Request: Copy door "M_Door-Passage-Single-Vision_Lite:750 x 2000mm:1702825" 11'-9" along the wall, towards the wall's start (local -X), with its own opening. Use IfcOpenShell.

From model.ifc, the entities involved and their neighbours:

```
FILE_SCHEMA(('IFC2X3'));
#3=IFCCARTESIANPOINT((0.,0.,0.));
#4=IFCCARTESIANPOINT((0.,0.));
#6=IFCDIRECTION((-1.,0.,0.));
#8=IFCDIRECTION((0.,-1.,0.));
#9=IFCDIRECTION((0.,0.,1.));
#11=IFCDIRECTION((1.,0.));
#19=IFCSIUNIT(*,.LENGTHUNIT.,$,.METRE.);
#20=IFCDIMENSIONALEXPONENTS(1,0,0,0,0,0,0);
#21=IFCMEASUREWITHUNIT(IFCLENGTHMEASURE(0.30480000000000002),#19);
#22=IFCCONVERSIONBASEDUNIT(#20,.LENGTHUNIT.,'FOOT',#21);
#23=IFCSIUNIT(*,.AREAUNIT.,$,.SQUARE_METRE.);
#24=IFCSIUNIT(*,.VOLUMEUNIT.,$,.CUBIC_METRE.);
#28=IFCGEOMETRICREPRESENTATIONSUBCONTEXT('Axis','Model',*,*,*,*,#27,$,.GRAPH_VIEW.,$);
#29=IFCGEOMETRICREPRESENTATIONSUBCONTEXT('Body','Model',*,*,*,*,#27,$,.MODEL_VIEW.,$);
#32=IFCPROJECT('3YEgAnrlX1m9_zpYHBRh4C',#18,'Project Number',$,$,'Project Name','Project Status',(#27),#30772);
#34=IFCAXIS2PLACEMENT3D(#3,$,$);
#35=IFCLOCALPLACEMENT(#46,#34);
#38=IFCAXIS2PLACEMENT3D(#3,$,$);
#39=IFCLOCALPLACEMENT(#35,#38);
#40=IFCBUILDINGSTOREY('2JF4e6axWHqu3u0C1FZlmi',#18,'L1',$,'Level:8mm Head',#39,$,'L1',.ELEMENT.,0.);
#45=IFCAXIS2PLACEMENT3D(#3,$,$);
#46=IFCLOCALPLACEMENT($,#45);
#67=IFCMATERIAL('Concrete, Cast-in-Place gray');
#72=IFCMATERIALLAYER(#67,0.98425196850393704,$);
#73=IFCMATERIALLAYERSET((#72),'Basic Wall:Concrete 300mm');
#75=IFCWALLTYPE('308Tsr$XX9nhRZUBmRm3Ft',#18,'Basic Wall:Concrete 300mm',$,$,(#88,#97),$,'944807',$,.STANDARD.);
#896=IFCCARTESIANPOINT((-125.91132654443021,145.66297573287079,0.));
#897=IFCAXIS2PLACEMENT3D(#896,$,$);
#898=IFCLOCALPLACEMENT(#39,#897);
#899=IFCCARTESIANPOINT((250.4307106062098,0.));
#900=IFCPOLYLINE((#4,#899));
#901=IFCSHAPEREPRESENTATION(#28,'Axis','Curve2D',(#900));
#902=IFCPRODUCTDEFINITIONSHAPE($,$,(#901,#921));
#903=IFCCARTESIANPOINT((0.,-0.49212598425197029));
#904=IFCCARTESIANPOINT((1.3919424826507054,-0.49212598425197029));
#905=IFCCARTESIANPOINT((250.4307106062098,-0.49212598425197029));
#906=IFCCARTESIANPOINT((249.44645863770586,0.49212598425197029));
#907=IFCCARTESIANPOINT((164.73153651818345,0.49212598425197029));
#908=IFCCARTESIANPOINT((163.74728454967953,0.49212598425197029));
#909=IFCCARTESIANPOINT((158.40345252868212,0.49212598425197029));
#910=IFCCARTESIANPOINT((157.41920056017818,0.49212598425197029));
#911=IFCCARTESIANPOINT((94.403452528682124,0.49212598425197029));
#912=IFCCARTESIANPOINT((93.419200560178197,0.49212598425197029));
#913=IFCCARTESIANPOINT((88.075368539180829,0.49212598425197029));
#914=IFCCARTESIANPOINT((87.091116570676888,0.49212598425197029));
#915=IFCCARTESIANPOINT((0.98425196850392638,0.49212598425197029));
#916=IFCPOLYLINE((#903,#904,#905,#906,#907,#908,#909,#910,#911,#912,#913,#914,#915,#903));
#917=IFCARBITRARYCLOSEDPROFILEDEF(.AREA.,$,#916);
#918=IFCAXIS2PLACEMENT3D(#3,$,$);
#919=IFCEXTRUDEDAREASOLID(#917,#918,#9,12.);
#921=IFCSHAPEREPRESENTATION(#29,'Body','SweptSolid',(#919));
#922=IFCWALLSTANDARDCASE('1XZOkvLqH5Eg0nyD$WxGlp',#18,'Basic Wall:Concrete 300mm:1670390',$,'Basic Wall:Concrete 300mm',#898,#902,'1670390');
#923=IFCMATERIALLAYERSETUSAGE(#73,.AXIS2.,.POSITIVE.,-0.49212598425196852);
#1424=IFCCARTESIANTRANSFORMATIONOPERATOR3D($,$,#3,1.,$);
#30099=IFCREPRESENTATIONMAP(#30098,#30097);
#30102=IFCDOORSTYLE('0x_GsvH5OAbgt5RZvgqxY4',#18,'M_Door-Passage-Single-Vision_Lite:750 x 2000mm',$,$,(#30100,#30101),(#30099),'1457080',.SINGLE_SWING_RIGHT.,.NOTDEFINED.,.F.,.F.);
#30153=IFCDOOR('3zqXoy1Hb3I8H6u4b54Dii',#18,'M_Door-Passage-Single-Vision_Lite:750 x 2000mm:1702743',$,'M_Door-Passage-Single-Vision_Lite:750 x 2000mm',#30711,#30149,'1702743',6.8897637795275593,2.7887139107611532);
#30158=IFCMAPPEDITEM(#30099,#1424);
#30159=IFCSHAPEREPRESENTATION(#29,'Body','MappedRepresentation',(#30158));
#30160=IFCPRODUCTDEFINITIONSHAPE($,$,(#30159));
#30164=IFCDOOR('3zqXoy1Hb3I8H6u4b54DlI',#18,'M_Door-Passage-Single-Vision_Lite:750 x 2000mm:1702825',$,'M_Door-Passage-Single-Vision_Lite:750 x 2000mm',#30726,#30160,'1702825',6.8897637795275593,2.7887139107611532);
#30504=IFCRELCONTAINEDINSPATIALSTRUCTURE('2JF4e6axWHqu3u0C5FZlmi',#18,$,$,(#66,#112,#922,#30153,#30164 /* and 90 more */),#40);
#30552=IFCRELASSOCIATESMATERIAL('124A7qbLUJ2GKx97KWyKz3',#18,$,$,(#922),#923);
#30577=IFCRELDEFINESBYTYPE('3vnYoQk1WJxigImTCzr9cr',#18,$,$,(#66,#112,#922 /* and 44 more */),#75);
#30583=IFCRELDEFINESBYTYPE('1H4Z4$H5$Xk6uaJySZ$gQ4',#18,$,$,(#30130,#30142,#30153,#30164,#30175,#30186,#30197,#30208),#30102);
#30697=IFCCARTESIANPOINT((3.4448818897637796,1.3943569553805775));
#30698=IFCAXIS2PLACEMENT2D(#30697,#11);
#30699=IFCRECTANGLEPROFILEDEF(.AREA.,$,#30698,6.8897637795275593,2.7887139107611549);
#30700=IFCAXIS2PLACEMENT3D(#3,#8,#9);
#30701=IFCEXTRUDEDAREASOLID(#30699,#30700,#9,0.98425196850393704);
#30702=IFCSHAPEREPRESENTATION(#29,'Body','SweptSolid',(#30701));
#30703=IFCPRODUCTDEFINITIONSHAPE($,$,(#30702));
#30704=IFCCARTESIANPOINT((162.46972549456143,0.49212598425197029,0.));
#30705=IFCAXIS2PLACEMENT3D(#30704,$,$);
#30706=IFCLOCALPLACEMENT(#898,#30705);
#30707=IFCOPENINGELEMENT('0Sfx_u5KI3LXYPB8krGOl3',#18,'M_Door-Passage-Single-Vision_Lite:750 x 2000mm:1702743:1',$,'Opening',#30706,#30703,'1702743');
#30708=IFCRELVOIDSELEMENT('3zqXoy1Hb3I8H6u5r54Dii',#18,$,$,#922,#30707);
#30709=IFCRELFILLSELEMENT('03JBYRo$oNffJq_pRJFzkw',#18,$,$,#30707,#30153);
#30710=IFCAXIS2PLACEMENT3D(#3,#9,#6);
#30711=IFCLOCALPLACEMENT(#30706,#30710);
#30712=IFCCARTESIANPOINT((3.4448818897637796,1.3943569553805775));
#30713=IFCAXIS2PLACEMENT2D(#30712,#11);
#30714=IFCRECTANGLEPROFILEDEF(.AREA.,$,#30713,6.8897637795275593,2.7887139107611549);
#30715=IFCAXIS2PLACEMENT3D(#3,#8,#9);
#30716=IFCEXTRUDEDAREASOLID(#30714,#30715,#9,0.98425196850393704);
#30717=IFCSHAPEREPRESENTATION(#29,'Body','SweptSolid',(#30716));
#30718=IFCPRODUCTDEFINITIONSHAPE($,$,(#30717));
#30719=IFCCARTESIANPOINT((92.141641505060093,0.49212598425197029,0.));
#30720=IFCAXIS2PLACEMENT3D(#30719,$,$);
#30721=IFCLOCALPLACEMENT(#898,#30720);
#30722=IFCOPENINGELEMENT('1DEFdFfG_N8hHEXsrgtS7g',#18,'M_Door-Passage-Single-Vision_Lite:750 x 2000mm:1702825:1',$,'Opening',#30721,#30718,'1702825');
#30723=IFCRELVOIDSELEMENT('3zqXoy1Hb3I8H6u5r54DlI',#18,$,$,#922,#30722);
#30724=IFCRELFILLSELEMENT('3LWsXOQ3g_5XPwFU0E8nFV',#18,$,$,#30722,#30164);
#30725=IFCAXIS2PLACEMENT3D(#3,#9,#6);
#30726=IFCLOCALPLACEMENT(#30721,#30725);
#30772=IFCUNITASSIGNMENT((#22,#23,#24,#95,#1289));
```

```python
import ifcopenshell
import ifcopenshell.api.feature
import ifcopenshell.api.geometry
import ifcopenshell.api.root
import ifcopenshell.geom
import ifcopenshell.util.element
import ifcopenshell.util.placement
import ifcopenshell.util.shape
import ifcopenshell.util.unit

model = ifcopenshell.open("model.ifc")
unit_scale = ifcopenshell.util.unit.calculate_unit_scale(model)
settings = ifcopenshell.geom.settings()


def volume(element):
    """Net volume in cubic metres, openings subtracted."""
    shape = ifcopenshell.geom.create_shape(settings, element)
    return ifcopenshell.util.shape.get_volume(shape.geometry)


def reuse_history(source, copy):
    """copy_class also copies each property set's owner history, people and application; keep the originals."""
    for rel in copy.IsDefinedBy:
        if rel.is_a("IfcRelDefinesByProperties") and (history := rel.RelatingPropertyDefinition.OwnerHistory):
            rel.RelatingPropertyDefinition.OwnerHistory = source.OwnerHistory
            ifcopenshell.util.element.remove_deep2(model, history)


door = model.by_id(30164)
opening = door.FillsVoids[0].RelatingOpeningElement
wall = opening.VoidsElements[0].RelatingBuildingElement
before = volume(wall)
shift = ifcopenshell.util.placement.get_local_placement(wall.ObjectPlacement)[:3, 0] * -141 * 0.0254 / unit_scale

# copy_class copies the void relationship, type, container and properties, but no geometry.
new_opening = ifcopenshell.api.root.copy_class(model, product=opening)
new_opening.Representation = ifcopenshell.util.element.copy_deep(
    model, opening.Representation, exclude=["IfcGeometricRepresentationContext", "IfcRepresentationMap"]
)
new_opening.Name = "M_Door-Passage-Single-Vision_Lite:750 x 2000mm"
new_opening.Tag = None
new_door = ifcopenshell.api.root.copy_class(model, product=door)
new_door.Representation = ifcopenshell.util.element.copy_deep(
    model, door.Representation, exclude=["IfcGeometricRepresentationContext", "IfcRepresentationMap"]
)
new_door.Name = "M_Door-Passage-Single-Vision_Lite:750 x 2000mm"
new_door.Tag = None
reuse_history(door, new_door)
fills = ifcopenshell.api.feature.add_filling(model, opening=new_opening, element=new_door)
fills.OwnerHistory = new_door.OwnerHistory  # required in IFC2X3

for old, new in ((opening, new_opening), (door, new_door)):
    matrix = ifcopenshell.util.placement.get_local_placement(old.ObjectPlacement)
    matrix[:3, 3] += shift
    ifcopenshell.api.geometry.edit_object_placement(model, product=new, matrix=matrix, is_si=False)

after = volume(wall)

print(f"wall volume {before:.3f} -> {after:.3f} m3")

model.write("model_updated.ifc")
```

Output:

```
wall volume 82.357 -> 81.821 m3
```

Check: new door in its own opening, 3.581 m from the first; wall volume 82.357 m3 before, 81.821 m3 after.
